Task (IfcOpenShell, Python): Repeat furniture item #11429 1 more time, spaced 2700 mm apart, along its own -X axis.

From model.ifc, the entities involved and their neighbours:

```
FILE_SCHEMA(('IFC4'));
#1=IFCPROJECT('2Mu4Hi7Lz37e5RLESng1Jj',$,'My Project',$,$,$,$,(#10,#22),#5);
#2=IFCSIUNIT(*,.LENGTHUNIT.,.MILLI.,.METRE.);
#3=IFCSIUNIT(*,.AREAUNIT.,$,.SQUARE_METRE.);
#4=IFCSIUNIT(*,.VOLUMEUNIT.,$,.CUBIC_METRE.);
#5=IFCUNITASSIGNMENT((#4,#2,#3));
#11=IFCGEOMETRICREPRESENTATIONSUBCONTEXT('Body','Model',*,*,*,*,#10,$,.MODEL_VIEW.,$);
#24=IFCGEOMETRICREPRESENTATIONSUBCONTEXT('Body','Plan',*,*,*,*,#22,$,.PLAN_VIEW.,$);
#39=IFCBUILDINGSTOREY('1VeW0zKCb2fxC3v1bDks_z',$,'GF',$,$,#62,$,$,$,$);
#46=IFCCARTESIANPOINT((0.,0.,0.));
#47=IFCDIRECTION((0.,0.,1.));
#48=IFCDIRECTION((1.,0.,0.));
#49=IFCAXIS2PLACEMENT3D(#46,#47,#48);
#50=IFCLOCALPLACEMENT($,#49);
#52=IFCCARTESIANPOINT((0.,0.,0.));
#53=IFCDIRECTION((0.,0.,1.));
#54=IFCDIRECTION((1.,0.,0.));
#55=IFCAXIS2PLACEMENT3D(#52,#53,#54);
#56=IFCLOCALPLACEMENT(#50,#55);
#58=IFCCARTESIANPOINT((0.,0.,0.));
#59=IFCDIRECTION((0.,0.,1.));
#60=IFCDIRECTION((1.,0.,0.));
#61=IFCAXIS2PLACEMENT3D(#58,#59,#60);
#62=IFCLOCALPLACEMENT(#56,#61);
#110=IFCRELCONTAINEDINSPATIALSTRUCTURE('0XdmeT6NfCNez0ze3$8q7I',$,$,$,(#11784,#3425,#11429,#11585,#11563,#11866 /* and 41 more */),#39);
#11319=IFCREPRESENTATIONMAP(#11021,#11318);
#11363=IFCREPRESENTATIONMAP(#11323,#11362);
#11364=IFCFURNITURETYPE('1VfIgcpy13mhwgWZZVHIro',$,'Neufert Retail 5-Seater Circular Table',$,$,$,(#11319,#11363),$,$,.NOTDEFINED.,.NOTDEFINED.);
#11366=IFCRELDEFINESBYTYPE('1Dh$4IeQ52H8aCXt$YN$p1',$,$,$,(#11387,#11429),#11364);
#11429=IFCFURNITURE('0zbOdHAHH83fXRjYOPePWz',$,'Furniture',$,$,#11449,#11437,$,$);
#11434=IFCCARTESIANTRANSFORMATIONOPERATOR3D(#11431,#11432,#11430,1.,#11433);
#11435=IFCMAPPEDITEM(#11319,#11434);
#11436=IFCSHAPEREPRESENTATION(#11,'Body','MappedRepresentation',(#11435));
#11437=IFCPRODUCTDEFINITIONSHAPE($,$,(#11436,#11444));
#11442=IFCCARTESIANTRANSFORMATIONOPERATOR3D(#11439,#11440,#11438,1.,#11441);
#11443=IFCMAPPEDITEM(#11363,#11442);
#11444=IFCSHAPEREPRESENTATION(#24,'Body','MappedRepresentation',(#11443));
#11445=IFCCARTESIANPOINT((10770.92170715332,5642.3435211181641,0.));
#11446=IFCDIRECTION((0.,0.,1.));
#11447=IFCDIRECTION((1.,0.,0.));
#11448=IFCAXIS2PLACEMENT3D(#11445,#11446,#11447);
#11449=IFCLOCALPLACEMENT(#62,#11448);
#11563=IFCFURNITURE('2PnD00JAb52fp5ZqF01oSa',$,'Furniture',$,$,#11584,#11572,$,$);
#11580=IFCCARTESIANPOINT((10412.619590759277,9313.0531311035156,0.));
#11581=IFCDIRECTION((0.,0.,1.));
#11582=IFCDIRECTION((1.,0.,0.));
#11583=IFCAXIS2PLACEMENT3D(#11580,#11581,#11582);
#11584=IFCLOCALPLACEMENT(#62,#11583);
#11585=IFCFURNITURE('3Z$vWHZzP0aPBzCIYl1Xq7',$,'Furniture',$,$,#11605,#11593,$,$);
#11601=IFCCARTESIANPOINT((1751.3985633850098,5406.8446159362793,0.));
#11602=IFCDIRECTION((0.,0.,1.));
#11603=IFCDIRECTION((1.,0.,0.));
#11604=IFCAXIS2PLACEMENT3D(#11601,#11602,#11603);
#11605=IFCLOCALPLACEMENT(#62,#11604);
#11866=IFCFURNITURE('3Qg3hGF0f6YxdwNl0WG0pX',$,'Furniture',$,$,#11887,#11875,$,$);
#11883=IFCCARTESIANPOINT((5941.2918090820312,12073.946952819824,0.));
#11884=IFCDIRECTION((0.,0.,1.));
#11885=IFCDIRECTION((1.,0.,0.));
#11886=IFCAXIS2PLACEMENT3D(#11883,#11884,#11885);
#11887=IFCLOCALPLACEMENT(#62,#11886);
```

```python
import ifcopenshell
import ifcopenshell.api.geometry
import ifcopenshell.api.root
import ifcopenshell.util.element
import ifcopenshell.util.placement

model = ifcopenshell.open("model.ifc")

source = model.by_id(11429)
base = ifcopenshell.util.placement.get_local_placement(source.ObjectPlacement)
step = -base[:3, 0] * 2700.0

for i in range(1, 2):
    copy = ifcopenshell.api.root.copy_class(model, product=source)
    copy.Representation = ifcopenshell.util.element.copy_deep(
        model, source.Representation, exclude=["IfcGeometricRepresentationContext", "IfcRepresentationMap"]
    )
    matrix = base.copy()
    matrix[:3, 3] += i * step
    print("added at", matrix[:3, 3].round(3) + 0.0)
    ifcopenshell.api.geometry.edit_object_placement(model, product=copy, matrix=matrix, is_si=False)

model.write("model_updated.ifc")
```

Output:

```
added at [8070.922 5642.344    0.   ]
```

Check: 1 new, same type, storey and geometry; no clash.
